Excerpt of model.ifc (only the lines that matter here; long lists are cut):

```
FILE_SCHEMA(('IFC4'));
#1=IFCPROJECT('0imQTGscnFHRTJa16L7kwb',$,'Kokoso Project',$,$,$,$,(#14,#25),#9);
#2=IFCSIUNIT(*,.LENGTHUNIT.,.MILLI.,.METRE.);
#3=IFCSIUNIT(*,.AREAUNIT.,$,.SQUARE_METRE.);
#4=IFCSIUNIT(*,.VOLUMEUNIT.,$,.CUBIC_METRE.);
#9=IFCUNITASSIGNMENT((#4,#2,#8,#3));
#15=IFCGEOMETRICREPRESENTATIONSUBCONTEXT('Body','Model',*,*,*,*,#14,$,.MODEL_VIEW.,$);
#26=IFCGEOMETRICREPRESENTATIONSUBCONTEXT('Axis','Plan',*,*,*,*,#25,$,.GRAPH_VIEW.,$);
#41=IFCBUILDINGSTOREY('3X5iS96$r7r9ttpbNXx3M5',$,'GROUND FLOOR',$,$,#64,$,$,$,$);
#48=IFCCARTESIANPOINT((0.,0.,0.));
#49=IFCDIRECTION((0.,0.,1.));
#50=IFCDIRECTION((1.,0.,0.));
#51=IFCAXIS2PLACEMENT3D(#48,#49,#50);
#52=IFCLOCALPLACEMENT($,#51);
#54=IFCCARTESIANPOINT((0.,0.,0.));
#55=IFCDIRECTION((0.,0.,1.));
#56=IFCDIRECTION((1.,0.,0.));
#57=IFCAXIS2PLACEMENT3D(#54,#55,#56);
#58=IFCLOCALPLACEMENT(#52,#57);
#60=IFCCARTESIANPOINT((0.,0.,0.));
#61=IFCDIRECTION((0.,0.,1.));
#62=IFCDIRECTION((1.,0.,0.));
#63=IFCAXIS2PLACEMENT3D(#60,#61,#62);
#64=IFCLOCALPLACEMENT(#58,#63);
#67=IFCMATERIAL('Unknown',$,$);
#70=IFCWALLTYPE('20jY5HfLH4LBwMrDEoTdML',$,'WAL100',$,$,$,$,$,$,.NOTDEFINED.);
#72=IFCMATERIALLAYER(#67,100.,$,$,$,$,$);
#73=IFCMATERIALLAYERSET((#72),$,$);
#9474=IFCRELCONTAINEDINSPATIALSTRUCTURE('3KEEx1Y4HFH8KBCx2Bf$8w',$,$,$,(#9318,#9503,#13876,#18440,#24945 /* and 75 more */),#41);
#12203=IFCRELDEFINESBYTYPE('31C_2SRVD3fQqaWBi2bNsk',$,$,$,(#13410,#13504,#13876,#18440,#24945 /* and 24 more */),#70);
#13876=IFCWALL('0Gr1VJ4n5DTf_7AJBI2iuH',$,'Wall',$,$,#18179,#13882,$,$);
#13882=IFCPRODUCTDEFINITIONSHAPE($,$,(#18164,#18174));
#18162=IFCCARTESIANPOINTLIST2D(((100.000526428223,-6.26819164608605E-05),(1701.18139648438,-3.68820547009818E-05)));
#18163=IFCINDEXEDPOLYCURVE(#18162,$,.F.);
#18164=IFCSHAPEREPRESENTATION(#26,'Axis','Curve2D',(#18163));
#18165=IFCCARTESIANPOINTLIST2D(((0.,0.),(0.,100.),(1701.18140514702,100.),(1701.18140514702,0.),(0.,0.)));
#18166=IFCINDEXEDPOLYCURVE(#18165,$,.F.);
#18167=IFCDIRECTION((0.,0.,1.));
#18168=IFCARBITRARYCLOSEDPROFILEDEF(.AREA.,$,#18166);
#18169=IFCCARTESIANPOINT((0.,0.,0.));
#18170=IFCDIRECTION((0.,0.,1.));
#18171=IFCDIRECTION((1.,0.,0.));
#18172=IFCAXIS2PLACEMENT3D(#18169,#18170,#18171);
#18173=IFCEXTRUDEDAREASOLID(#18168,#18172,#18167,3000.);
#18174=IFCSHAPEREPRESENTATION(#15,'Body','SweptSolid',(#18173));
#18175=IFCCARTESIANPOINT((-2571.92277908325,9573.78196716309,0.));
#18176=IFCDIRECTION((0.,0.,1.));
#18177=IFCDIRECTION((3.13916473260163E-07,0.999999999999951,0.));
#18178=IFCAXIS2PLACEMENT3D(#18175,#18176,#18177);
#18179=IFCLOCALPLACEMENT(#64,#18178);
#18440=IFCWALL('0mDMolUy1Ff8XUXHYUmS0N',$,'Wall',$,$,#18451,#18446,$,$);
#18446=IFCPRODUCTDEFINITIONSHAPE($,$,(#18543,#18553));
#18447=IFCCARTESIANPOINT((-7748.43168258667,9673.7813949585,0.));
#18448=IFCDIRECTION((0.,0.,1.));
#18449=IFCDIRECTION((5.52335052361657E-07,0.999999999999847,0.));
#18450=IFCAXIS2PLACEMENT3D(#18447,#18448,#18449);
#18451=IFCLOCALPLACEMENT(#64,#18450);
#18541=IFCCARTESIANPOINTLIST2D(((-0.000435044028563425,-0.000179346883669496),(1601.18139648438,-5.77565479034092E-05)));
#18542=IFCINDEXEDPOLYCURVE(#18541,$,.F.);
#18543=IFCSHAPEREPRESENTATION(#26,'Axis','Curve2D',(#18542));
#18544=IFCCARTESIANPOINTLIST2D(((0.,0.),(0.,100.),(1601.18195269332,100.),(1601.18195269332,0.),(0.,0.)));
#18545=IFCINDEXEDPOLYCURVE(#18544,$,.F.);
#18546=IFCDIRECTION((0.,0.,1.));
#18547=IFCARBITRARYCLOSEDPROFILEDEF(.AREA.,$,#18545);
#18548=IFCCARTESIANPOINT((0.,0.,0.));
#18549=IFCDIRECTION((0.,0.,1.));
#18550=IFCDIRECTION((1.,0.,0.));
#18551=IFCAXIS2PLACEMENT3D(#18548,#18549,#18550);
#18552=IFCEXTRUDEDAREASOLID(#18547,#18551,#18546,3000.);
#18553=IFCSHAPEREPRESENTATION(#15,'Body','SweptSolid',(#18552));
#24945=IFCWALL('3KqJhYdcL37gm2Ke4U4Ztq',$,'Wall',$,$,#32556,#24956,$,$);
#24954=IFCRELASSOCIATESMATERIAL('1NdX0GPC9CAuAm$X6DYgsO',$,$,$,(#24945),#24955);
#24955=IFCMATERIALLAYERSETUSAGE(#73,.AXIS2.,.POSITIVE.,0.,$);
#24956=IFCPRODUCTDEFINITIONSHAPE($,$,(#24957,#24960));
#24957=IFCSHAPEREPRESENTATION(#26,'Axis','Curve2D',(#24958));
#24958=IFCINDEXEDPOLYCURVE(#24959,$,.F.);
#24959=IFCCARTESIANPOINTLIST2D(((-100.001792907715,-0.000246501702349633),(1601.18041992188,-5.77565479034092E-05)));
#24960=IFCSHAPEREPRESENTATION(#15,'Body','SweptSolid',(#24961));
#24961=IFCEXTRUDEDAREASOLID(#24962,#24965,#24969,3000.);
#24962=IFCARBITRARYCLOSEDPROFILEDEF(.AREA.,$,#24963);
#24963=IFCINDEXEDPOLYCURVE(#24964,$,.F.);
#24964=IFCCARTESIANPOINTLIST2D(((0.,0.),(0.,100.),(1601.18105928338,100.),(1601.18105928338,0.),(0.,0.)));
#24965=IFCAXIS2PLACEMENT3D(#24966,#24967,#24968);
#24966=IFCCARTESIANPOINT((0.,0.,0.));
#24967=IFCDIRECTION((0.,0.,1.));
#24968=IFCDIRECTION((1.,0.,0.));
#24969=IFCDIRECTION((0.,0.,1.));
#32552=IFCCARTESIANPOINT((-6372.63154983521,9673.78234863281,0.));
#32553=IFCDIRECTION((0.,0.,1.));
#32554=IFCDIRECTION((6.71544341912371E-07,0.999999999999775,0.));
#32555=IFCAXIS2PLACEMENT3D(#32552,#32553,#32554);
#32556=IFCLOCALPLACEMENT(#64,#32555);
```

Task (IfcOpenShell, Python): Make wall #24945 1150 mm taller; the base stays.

```python
import ifcopenshell
import ifcopenshell.geom
import ifcopenshell.util.representation
import ifcopenshell.util.shape
import ifcopenshell.util.unit

model = ifcopenshell.open("model.ifc")
unit_scale = ifcopenshell.util.unit.calculate_unit_scale(model)
settings = ifcopenshell.geom.settings()


def volume(element):
    """Net volume in cubic metres, openings subtracted."""
    shape = ifcopenshell.geom.create_shape(settings, element)
    return ifcopenshell.util.shape.get_volume(shape.geometry)


wall = model.by_id(24945)
before = volume(wall)

body = ifcopenshell.util.representation.get_representation(wall, "Model", "Body")
solid = body.Items[0]
old_height = solid.Depth
solid.Depth += 1.15 / unit_scale
after = volume(wall)

print(f"height {old_height:g} -> {solid.Depth:g}, volume {before:.3f} -> {after:.3f} m3")

model.write("model_updated.ifc")
```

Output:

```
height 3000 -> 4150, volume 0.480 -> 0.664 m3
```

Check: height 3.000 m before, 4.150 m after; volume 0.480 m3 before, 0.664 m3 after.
